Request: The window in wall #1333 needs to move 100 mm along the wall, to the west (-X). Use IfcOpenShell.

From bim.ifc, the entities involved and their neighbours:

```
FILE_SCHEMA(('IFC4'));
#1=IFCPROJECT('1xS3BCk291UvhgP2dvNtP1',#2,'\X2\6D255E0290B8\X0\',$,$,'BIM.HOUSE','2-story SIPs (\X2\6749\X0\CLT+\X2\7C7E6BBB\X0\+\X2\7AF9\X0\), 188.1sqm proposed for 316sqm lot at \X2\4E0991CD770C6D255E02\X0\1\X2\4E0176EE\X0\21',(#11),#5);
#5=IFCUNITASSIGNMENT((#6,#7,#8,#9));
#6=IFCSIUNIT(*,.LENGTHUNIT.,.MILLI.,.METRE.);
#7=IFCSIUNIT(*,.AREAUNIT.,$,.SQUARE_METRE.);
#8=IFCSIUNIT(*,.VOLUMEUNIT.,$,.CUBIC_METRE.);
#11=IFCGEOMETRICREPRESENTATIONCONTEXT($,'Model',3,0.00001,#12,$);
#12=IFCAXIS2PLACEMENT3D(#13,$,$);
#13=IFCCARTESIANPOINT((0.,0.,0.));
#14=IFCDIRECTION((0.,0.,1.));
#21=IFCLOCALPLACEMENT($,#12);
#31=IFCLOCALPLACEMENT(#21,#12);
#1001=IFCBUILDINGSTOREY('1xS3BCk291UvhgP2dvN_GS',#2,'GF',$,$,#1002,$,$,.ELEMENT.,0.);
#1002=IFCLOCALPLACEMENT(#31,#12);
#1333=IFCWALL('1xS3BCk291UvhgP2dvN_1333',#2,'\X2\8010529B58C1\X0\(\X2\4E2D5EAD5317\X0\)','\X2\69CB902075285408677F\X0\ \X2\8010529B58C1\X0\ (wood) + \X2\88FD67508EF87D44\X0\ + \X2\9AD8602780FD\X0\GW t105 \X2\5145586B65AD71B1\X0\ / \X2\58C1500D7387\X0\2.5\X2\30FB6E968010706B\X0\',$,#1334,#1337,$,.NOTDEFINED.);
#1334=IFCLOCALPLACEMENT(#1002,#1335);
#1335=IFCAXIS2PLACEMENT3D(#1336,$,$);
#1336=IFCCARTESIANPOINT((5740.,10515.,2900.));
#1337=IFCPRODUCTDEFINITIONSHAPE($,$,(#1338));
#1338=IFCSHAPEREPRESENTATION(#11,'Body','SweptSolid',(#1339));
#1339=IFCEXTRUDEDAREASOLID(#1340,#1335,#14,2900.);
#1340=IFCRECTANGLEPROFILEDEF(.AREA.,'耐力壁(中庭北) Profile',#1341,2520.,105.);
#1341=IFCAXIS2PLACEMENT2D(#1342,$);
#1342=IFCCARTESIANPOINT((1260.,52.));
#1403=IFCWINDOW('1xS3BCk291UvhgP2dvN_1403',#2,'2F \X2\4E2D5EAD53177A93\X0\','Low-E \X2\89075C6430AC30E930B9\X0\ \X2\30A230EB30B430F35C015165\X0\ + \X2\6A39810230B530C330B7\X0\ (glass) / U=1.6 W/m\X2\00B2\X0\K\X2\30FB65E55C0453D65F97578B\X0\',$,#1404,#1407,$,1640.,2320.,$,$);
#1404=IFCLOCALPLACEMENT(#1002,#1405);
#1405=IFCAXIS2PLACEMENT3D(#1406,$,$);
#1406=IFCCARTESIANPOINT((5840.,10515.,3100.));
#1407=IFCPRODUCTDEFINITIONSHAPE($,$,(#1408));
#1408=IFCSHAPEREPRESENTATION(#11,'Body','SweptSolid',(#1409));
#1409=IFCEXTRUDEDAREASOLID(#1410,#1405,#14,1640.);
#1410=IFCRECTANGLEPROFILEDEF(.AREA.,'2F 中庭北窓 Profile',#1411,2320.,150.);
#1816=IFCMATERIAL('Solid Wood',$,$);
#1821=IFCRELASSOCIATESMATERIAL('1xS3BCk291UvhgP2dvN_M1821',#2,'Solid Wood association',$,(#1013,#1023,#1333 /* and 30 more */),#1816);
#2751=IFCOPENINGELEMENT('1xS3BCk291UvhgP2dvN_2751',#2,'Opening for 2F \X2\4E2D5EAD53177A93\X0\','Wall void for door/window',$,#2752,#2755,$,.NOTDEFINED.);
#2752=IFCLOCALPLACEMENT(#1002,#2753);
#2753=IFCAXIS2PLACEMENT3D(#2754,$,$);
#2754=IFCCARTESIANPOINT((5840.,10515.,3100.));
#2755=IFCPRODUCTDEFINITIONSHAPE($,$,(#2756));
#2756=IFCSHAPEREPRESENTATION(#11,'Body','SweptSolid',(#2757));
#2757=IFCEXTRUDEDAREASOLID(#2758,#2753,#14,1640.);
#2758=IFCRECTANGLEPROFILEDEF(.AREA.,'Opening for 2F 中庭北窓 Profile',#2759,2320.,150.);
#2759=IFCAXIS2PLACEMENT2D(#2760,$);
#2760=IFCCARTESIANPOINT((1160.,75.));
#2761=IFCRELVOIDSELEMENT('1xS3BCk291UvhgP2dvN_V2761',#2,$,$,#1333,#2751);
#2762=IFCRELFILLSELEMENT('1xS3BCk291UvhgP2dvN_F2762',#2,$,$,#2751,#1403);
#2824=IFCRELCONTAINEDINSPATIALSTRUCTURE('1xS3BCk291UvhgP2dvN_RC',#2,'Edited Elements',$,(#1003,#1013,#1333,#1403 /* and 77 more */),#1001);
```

```python
import ifcopenshell
import ifcopenshell.api.geometry
import ifcopenshell.util.placement
import ifcopenshell.util.unit

model = ifcopenshell.open("bim.ifc")
unit_scale = ifcopenshell.util.unit.calculate_unit_scale(model)

window = model.by_guid("1xS3BCk291UvhgP2dvN_1403")
opening = window.FillsVoids[0].RelatingOpeningElement
wall = opening.VoidsElements[0].RelatingBuildingElement

wall_matrix = ifcopenshell.util.placement.get_local_placement(wall.ObjectPlacement)
shift = wall_matrix[:3, 0] * -0.1 / unit_scale
before = ifcopenshell.util.placement.get_local_placement(window.ObjectPlacement)[:3, 3].copy()

# The window is not placed relative to its opening, so move both.
for product in (opening, window):
    matrix = ifcopenshell.util.placement.get_local_placement(product.ObjectPlacement)
    matrix[:3, 3] += shift
    ifcopenshell.api.geometry.edit_object_placement(model, product=product, matrix=matrix, is_si=False)

after = ifcopenshell.util.placement.get_local_placement(window.ObjectPlacement)[:3, 3]
print("window moved by", (after - before).round(3) + 0.0)

model.write("bim_edited.ifc")
```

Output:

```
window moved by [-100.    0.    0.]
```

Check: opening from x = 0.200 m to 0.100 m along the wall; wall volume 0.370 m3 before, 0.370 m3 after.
